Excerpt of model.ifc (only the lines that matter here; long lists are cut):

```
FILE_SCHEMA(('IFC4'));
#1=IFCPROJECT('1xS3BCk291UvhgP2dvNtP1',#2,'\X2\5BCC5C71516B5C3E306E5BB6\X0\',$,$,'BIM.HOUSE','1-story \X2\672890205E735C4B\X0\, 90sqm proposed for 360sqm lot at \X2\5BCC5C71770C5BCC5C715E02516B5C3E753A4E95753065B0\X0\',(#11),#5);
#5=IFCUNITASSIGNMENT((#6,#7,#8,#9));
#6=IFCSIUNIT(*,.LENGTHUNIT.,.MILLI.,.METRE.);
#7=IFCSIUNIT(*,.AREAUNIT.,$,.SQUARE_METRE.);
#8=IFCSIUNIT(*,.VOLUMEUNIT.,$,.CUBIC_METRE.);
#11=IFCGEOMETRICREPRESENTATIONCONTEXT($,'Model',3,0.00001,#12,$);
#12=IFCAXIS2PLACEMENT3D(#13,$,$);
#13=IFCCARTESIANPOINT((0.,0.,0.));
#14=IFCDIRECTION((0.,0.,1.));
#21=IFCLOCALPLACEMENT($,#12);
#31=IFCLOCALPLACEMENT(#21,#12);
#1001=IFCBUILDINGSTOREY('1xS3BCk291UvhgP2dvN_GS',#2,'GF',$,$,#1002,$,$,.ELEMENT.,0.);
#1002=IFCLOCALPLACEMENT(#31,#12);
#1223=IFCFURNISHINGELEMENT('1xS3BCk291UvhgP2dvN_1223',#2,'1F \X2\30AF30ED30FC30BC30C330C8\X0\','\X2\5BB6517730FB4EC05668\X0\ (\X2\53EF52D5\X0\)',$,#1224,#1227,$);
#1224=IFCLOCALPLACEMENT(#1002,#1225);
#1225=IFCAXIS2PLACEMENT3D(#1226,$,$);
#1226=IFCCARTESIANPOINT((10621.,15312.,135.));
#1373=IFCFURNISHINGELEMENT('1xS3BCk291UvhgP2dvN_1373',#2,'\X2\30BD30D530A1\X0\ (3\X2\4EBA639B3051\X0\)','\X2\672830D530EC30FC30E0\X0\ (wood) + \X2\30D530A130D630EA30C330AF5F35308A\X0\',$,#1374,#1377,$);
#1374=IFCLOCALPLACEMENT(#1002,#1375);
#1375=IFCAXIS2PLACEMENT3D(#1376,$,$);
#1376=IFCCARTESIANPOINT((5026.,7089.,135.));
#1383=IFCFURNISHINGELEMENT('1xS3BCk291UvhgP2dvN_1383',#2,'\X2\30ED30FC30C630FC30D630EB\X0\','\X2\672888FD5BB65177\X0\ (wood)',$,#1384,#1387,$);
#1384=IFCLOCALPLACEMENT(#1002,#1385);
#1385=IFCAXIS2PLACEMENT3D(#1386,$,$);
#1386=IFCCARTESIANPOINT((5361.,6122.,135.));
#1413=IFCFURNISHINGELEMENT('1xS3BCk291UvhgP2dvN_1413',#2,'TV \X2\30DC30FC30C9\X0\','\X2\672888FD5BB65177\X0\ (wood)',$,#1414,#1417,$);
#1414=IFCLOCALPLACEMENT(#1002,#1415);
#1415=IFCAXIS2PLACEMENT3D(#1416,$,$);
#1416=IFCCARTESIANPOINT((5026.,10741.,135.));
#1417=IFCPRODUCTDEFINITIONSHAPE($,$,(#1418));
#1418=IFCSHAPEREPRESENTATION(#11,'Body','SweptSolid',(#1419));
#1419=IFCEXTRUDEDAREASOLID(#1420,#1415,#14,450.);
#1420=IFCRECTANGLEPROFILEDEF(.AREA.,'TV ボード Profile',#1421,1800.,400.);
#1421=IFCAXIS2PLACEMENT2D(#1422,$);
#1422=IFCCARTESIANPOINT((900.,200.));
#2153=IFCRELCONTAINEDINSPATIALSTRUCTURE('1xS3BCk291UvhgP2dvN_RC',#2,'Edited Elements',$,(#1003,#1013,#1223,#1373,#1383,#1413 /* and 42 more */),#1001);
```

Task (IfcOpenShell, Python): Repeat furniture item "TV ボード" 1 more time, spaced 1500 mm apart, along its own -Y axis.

```python
import ifcopenshell
import ifcopenshell.api.geometry
import ifcopenshell.api.root
import ifcopenshell.util.element
import ifcopenshell.util.placement
import ifcopenshell.util.unit

model = ifcopenshell.open("model.ifc")
unit_scale = ifcopenshell.util.unit.calculate_unit_scale(model)


def reuse_history(source, copy):
    """copy_class also copies each property set's owner history, people and application; keep the originals."""
    for rel in copy.IsDefinedBy:
        if rel.is_a("IfcRelDefinesByProperties") and (history := rel.RelatingPropertyDefinition.OwnerHistory):
            rel.RelatingPropertyDefinition.OwnerHistory = source.OwnerHistory
            ifcopenshell.util.element.remove_deep2(model, history)


source = model.by_id(1413)
base = ifcopenshell.util.placement.get_local_placement(source.ObjectPlacement)
step = -base[:3, 1] * 1.5 / unit_scale

for i in range(1, 2):
    copy = ifcopenshell.api.root.copy_class(model, product=source)
    copy.Representation = ifcopenshell.util.element.copy_deep(
        model, source.Representation, exclude=["IfcGeometricRepresentationContext", "IfcRepresentationMap"]
    )
    reuse_history(source, copy)
    matrix = base.copy()
    matrix[:3, 3] += i * step
    print("added at", matrix[:3, 3].round(3) + 0.0)
    ifcopenshell.api.geometry.edit_object_placement(model, product=copy, matrix=matrix, is_si=False)

model.write("model_v2.ifc")
```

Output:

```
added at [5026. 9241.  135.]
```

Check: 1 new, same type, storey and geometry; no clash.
